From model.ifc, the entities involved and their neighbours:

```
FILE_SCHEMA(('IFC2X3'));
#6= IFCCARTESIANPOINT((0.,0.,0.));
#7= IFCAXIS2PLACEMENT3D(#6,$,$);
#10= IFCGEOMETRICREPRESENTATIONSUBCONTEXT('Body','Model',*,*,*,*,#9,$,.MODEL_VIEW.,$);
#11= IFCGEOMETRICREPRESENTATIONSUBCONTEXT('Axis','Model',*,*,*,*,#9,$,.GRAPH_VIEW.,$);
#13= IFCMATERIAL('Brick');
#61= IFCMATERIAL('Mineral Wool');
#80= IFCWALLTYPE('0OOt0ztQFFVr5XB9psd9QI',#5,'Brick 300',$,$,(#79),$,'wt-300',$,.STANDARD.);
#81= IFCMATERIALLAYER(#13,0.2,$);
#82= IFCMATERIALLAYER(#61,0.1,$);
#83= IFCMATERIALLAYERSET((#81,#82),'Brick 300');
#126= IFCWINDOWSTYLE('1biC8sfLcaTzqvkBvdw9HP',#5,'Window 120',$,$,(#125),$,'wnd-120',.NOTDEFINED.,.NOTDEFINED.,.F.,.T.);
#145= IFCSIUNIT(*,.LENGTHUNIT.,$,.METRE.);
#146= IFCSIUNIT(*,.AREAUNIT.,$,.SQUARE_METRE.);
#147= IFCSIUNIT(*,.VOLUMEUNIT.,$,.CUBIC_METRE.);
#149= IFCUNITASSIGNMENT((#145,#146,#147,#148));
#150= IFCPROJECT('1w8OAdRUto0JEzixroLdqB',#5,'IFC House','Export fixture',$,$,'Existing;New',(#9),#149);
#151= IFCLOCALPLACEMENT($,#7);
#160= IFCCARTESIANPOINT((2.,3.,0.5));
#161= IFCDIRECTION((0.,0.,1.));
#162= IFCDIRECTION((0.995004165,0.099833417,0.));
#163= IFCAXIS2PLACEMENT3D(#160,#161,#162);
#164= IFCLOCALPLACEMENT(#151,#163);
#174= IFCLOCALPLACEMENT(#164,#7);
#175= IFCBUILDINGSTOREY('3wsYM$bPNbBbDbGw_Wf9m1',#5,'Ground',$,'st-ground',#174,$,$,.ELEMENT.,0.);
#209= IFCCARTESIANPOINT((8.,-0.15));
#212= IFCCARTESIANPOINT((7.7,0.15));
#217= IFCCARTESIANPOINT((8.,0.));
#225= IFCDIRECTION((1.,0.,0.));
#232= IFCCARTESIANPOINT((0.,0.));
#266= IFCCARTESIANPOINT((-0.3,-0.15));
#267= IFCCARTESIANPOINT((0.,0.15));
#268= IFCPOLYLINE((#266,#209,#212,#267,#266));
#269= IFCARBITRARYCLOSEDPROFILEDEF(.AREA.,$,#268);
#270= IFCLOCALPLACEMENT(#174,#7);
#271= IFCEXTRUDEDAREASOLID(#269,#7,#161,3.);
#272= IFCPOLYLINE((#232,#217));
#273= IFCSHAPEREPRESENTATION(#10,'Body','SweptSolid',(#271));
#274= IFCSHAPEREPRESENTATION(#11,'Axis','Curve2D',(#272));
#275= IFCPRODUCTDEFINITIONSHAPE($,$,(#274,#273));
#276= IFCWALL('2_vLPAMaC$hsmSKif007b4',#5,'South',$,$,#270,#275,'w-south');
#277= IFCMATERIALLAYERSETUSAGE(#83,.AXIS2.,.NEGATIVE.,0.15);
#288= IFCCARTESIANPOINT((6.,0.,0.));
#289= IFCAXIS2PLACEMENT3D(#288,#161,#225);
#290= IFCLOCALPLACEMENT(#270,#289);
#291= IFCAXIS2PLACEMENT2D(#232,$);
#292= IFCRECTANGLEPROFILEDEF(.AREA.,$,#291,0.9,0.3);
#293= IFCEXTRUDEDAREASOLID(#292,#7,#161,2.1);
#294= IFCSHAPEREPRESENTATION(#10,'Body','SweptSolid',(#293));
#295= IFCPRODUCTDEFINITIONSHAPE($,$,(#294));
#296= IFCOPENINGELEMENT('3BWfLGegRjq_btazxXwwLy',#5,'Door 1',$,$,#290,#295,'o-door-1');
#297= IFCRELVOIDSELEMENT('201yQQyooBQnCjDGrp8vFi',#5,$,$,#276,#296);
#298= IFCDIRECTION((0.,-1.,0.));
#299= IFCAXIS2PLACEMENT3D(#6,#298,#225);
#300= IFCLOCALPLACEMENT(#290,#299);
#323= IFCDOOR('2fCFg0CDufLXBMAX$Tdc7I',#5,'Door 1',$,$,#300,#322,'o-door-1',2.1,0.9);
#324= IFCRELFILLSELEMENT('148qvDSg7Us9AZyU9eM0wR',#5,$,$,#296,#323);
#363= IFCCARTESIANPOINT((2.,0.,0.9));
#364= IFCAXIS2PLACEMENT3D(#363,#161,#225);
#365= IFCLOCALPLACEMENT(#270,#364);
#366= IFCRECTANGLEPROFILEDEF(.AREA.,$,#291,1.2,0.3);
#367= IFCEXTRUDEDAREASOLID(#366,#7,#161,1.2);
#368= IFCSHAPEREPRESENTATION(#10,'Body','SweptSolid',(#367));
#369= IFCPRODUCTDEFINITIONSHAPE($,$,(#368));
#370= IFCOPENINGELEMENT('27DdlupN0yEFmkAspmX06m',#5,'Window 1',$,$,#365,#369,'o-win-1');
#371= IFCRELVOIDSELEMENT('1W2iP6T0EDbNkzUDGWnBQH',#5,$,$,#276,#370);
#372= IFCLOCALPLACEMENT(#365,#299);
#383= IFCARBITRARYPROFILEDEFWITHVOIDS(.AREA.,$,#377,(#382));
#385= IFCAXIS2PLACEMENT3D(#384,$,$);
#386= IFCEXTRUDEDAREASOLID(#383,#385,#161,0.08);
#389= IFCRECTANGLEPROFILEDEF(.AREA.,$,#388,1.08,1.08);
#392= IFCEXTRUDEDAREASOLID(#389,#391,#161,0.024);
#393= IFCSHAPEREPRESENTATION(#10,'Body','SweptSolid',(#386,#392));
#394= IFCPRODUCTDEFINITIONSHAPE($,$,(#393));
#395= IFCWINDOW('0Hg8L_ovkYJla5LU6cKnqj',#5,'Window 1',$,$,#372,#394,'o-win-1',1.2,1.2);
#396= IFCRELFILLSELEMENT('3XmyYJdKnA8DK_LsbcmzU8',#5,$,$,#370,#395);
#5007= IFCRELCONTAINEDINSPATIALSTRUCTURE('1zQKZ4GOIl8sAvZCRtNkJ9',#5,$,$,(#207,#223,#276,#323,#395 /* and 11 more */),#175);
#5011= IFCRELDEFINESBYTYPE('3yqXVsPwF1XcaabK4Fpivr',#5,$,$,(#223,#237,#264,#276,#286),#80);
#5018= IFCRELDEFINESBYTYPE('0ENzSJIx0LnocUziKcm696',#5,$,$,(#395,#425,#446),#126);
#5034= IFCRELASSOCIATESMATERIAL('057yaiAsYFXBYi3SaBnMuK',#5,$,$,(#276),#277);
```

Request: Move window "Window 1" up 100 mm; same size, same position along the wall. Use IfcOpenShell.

```python
import numpy as np
import ifcopenshell
import ifcopenshell.api.geometry
import ifcopenshell.util.placement
import ifcopenshell.util.unit

model = ifcopenshell.open("model.ifc")
unit_scale = ifcopenshell.util.unit.calculate_unit_scale(model)

window = model.by_guid("0Hg8L_ovkYJla5LU6cKnqj")
opening = window.FillsVoids[0].RelatingOpeningElement
dz = 0.1 / unit_scale

shift = np.array([0.0, 0.0, dz])
# The window is placed relative to its opening, so it follows when the opening moves.
matrix = ifcopenshell.util.placement.get_local_placement(opening.ObjectPlacement)
matrix[:3, 3] += shift
ifcopenshell.api.geometry.edit_object_placement(
    model, product=opening, matrix=matrix, is_si=False, should_transform_children=True
)

print(f"moved by {dz * unit_scale:+.3f} m")

model.write("model-out.ifc")
```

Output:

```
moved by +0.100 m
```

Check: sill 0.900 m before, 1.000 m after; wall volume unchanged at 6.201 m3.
